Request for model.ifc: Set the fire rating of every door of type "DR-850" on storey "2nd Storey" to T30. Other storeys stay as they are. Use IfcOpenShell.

First a look at what the model holds.

```python
import ifcopenshell
import ifcopenshell.util.element

model = ifcopenshell.open("model.ifc")
print(model.schema)
storey = next(s for s in model.by_type("IfcBuildingStorey") if s.Name == "2nd Storey")
doors = [e for e in ifcopenshell.util.element.get_decomposition(storey) if e.is_a("IfcDoor")]
seen = {}
for e in doors:
    element_type = ifcopenshell.util.element.get_type(e)
    key = (element_type.Name if element_type != e and element_type else None, ifcopenshell.util.element.get_pset(e, "Pset_DoorCommon", "FireRating"))
    seen[key] = seen.get(key, 0) + 1
for (name, value), count in sorted(seen.items(), key=str):
    print(count, "x", name, "|", value)
```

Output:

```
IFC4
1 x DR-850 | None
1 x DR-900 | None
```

```python
import ifcopenshell
import ifcopenshell.api.pset
import ifcopenshell.util.element

model = ifcopenshell.open("model.ifc")

storey = next(s for s in model.by_type("IfcBuildingStorey") if s.Name == "2nd Storey")
doors = [e for e in ifcopenshell.util.element.get_decomposition(storey) if e.is_a("IfcDoor")]

count = 0
for e in doors:
    element_type = ifcopenshell.util.element.get_type(e)
    if element_type in (None, e) or element_type.Name != "DR-850":
        continue
    # add_pset returns the element's existing set when there is one.
    pset = ifcopenshell.api.pset.add_pset(model, product=e, name="Pset_DoorCommon")
    ifcopenshell.api.pset.edit_pset(model, pset=pset, properties={"FireRating": "T30"})
    count += 1

print(count, "doors updated")

model.write("model-out.ifc")
```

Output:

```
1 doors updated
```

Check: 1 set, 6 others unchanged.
